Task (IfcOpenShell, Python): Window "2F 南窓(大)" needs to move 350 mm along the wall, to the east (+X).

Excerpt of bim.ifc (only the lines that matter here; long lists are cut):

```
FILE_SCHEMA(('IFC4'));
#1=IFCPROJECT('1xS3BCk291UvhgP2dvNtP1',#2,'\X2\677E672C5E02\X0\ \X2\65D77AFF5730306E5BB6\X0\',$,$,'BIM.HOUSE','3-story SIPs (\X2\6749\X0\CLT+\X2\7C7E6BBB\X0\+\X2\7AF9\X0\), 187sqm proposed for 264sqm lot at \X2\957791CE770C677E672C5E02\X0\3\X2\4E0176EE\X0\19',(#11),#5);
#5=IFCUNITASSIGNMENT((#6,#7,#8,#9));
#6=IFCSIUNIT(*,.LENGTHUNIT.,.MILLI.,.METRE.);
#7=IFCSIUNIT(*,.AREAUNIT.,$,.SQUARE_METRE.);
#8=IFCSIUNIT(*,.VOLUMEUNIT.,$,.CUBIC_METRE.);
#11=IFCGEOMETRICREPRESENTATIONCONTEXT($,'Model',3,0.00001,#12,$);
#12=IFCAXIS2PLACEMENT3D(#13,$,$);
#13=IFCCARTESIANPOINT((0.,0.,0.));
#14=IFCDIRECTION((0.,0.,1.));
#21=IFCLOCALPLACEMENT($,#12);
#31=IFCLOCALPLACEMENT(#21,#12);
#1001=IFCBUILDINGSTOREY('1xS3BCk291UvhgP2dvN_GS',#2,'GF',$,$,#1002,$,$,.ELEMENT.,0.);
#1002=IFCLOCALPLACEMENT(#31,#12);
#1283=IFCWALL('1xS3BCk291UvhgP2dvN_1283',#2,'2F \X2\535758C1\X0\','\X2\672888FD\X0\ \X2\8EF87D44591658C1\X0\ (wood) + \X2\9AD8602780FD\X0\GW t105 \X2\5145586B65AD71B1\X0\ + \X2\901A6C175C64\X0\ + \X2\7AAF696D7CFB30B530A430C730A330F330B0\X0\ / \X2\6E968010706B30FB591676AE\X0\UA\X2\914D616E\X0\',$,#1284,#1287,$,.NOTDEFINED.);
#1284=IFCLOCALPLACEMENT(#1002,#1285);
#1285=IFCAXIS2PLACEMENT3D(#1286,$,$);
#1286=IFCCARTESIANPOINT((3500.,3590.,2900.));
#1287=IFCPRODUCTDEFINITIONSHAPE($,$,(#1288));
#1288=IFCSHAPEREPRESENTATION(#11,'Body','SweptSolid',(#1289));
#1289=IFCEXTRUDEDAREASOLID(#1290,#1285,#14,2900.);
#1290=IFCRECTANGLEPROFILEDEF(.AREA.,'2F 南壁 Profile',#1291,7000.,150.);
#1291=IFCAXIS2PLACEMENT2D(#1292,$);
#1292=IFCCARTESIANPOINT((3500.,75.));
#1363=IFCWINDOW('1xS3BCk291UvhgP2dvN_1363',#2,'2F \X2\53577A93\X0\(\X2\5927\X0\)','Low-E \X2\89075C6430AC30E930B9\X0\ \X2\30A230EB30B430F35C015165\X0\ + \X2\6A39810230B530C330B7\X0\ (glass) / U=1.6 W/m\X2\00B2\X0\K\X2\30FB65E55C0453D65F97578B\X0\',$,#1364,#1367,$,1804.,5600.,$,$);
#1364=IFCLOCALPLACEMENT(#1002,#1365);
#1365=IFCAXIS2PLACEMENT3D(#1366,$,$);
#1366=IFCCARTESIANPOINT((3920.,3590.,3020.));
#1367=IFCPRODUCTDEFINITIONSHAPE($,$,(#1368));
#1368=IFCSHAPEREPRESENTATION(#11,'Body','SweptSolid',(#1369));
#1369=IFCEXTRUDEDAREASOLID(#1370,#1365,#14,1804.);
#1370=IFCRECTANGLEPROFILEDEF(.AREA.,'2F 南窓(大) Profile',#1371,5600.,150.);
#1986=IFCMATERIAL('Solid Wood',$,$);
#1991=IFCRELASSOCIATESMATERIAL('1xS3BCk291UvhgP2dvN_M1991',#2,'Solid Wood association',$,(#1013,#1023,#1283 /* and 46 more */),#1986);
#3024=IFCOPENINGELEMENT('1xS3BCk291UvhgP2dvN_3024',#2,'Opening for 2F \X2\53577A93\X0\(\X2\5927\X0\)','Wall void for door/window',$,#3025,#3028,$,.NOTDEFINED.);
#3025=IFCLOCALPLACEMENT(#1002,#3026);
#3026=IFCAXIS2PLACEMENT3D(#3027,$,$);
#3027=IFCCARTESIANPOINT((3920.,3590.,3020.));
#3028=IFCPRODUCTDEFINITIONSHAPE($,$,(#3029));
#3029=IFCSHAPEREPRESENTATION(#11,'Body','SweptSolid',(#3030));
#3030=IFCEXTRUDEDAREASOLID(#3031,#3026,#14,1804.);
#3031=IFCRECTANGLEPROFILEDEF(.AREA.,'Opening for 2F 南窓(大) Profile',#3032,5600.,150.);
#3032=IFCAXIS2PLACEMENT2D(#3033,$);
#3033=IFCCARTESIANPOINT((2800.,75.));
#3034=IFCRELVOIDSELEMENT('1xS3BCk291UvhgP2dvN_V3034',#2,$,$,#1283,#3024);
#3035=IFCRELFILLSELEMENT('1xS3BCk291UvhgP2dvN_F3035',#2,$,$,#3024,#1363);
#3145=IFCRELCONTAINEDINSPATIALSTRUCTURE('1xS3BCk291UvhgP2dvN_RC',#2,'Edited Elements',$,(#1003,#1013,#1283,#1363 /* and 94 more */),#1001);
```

```python
import ifcopenshell
import ifcopenshell.api.geometry
import ifcopenshell.util.placement

model = ifcopenshell.open("bim.ifc")

window = model.by_guid("1xS3BCk291UvhgP2dvN_1363")
opening = window.FillsVoids[0].RelatingOpeningElement
wall = opening.VoidsElements[0].RelatingBuildingElement

wall_matrix = ifcopenshell.util.placement.get_local_placement(wall.ObjectPlacement)
shift = wall_matrix[:3, 0] * 350.0
before = ifcopenshell.util.placement.get_local_placement(window.ObjectPlacement)[:3, 3].copy()

# The window is not placed relative to its opening, so move both.
for product in (opening, window):
    matrix = ifcopenshell.util.placement.get_local_placement(product.ObjectPlacement)
    matrix[:3, 3] += shift
    ifcopenshell.api.geometry.edit_object_placement(model, product=product, matrix=matrix, is_si=False)

after = ifcopenshell.util.placement.get_local_placement(window.ObjectPlacement)[:3, 3]
print("window moved by", (after - before).round(3) + 0.0)

model.write("bim_rev.ifc")
```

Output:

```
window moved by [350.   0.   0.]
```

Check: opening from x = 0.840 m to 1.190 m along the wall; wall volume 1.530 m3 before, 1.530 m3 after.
